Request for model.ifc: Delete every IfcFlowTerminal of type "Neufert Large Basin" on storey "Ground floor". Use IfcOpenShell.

First a look at what the model holds.

```python
import ifcopenshell
import ifcopenshell.util.element

model = ifcopenshell.open("model.ifc")
print(model.schema)
storey = next(s for s in model.by_type("IfcBuildingStorey") if s.Name == "Ground floor")
terminals = [e for e in ifcopenshell.util.element.get_decomposition(storey) if e.is_a("IfcFlowTerminal")]
seen = {}
for e in terminals:
    element_type = ifcopenshell.util.element.get_type(e)
    name = element_type.Name if element_type not in (None, e) else None
    seen[name] = seen.get(name, 0) + 1
for name, count in sorted(seen.items(), key=str):
    print(count, "x", name)
```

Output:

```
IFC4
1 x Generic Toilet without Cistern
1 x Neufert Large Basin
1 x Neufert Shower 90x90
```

```python
import ifcopenshell
import ifcopenshell.api.root
import ifcopenshell.util.element

model = ifcopenshell.open("model.ifc")

storey = next(s for s in model.by_type("IfcBuildingStorey") if s.Name == "Ground floor")
terminals = [e for e in ifcopenshell.util.element.get_decomposition(storey) if e.is_a("IfcFlowTerminal")]
targets = [e for e in terminals if (t := ifcopenshell.util.element.get_type(e)) not in (None, e) and t.Name == "Neufert Large Basin"]

for e in targets:
    ifcopenshell.api.root.remove_product(model, product=e)
print(len(targets), "removed")

model.write("model-out.ifc")
```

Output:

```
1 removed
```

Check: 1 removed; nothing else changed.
